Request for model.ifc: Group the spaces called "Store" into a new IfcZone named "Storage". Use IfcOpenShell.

First a look at what the model holds.

```python
import ifcopenshell

model = ifcopenshell.open("model.ifc")
print(model.schema)
seen = {}
for space in model.by_type("IfcSpace"):
    seen[space.LongName] = seen.get(space.LongName, 0) + 1
for name, count in sorted(seen.items(), key=str):
    print(count, "x", name)
print("zones:", [z.Name for z in model.by_type("IfcZone")][:20])
```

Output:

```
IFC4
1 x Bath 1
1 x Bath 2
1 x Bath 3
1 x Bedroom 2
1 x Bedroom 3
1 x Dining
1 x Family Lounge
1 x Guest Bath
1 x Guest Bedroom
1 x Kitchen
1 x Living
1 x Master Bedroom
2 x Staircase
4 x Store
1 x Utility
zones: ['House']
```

```python
import ifcopenshell
import ifcopenshell.api.group
import ifcopenshell.api.root

model = ifcopenshell.open("model.ifc")

names = {"Store"}
spaces = [s for s in model.by_type("IfcSpace") if s.LongName in names]

zone = ifcopenshell.api.root.create_entity(model, ifc_class="IfcZone", name="Storage")
ifcopenshell.api.group.assign_group(model, products=spaces, group=zone)
print(len(spaces), "spaces in", zone.Name)

model.write("model_rev.ifc")
```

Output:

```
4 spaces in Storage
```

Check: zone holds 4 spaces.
